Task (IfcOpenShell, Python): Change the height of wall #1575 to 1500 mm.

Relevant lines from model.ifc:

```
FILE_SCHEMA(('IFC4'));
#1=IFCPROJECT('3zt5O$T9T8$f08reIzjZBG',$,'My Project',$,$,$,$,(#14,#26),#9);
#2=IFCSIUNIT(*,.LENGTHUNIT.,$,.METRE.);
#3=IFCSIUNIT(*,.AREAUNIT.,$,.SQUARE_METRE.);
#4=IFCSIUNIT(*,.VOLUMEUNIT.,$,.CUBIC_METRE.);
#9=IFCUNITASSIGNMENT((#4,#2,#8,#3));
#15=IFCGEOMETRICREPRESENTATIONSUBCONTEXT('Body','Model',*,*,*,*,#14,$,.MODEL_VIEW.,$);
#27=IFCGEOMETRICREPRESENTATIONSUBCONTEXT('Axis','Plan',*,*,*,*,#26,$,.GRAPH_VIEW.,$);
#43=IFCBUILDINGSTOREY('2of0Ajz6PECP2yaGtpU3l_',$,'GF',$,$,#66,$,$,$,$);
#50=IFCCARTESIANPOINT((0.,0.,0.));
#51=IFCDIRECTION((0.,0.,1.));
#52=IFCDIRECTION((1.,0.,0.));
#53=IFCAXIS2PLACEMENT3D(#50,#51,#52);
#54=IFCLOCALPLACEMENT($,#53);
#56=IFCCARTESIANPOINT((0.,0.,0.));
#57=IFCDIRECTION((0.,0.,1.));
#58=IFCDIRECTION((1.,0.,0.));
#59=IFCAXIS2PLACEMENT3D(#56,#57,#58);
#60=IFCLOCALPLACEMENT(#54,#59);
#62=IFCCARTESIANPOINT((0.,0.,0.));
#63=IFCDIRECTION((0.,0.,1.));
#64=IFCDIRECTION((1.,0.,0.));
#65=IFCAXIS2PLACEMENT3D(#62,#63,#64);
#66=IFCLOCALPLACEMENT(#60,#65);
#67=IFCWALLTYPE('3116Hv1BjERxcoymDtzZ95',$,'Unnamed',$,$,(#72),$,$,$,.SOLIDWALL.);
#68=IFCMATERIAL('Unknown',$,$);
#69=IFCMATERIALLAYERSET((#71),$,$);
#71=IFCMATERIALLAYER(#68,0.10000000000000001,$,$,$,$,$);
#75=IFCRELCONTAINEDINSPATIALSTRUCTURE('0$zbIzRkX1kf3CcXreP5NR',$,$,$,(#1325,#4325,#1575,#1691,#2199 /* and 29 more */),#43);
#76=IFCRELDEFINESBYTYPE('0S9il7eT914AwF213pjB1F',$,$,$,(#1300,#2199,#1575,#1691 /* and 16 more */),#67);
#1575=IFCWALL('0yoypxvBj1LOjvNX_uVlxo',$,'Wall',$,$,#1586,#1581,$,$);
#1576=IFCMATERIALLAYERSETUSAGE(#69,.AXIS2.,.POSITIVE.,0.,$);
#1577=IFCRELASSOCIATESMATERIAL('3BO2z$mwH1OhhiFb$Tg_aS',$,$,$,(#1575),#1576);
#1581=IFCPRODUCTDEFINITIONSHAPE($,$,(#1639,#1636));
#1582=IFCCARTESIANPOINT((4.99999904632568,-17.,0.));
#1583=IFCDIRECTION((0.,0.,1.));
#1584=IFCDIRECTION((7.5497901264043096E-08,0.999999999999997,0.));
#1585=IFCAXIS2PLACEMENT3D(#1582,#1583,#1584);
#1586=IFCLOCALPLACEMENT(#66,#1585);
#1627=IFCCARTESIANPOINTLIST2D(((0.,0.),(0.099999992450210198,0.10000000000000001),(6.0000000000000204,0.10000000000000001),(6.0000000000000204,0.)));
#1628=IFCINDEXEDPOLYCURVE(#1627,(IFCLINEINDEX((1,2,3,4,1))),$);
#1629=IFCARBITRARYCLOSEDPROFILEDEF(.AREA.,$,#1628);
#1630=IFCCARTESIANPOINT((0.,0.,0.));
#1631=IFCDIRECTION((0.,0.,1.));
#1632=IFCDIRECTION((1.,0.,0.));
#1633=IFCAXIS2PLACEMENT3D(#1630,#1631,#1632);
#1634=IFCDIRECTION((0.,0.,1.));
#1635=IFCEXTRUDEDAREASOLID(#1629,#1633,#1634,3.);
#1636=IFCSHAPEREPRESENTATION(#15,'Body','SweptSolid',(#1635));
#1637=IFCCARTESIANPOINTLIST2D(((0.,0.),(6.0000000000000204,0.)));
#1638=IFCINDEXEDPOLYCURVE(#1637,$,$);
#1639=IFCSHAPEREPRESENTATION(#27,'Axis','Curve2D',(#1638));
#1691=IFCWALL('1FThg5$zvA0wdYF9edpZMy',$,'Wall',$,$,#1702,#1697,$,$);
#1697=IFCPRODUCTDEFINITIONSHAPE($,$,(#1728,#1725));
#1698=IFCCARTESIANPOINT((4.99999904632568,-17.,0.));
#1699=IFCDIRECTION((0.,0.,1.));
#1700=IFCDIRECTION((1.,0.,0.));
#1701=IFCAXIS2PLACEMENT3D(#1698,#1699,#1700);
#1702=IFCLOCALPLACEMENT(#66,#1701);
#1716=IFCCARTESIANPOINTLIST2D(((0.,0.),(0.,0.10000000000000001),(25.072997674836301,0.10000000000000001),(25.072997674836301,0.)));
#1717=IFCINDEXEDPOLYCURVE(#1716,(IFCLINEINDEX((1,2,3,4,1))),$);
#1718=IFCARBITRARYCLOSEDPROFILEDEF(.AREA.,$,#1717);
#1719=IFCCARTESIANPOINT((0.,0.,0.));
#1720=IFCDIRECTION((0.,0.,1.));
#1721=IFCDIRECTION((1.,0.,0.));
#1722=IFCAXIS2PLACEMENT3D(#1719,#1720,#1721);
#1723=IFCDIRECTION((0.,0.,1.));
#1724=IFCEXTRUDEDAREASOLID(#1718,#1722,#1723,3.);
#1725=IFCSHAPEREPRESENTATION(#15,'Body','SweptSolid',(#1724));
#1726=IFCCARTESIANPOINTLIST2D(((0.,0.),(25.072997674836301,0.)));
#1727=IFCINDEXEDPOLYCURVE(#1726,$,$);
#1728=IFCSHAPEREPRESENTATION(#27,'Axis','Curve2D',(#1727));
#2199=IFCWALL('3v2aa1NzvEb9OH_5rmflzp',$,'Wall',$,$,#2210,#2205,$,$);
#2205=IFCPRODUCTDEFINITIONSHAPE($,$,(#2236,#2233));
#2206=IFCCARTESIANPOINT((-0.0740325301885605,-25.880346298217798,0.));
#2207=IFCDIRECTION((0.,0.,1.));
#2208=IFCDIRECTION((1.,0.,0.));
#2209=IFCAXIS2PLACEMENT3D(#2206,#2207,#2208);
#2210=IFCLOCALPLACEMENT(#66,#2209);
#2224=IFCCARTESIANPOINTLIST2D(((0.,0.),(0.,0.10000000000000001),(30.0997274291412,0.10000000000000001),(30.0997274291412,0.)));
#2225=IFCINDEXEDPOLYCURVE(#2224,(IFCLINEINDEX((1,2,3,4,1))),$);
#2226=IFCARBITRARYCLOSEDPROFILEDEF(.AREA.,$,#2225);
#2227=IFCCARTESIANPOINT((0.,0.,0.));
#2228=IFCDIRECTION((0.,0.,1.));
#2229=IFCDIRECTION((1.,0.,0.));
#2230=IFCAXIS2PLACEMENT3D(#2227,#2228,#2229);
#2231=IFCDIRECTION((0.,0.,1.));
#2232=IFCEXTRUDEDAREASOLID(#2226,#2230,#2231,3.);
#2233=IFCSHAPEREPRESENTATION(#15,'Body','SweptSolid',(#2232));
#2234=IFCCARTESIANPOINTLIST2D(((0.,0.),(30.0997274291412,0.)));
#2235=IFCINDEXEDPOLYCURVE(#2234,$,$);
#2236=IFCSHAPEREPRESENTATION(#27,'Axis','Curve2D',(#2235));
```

```python
import ifcopenshell
import ifcopenshell.geom
import ifcopenshell.util.representation
import ifcopenshell.util.shape

model = ifcopenshell.open("model.ifc")
settings = ifcopenshell.geom.settings()


def volume(element):
    """Net volume in cubic metres, openings subtracted."""
    shape = ifcopenshell.geom.create_shape(settings, element)
    return ifcopenshell.util.shape.get_volume(shape.geometry)


wall = model.by_guid("0yoypxvBj1LOjvNX_uVlxo")
before = volume(wall)

body = ifcopenshell.util.representation.get_representation(wall, "Model", "Body")
solid = body.Items[0]
old_height = solid.Depth
solid.Depth = 1.5
after = volume(wall)

print(f"height {old_height:g} -> {solid.Depth:g}, volume {before:.3f} -> {after:.3f} m3")

model.write("model_v2.ifc")
```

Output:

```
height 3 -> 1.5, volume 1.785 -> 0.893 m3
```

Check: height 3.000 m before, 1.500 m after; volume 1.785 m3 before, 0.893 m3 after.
